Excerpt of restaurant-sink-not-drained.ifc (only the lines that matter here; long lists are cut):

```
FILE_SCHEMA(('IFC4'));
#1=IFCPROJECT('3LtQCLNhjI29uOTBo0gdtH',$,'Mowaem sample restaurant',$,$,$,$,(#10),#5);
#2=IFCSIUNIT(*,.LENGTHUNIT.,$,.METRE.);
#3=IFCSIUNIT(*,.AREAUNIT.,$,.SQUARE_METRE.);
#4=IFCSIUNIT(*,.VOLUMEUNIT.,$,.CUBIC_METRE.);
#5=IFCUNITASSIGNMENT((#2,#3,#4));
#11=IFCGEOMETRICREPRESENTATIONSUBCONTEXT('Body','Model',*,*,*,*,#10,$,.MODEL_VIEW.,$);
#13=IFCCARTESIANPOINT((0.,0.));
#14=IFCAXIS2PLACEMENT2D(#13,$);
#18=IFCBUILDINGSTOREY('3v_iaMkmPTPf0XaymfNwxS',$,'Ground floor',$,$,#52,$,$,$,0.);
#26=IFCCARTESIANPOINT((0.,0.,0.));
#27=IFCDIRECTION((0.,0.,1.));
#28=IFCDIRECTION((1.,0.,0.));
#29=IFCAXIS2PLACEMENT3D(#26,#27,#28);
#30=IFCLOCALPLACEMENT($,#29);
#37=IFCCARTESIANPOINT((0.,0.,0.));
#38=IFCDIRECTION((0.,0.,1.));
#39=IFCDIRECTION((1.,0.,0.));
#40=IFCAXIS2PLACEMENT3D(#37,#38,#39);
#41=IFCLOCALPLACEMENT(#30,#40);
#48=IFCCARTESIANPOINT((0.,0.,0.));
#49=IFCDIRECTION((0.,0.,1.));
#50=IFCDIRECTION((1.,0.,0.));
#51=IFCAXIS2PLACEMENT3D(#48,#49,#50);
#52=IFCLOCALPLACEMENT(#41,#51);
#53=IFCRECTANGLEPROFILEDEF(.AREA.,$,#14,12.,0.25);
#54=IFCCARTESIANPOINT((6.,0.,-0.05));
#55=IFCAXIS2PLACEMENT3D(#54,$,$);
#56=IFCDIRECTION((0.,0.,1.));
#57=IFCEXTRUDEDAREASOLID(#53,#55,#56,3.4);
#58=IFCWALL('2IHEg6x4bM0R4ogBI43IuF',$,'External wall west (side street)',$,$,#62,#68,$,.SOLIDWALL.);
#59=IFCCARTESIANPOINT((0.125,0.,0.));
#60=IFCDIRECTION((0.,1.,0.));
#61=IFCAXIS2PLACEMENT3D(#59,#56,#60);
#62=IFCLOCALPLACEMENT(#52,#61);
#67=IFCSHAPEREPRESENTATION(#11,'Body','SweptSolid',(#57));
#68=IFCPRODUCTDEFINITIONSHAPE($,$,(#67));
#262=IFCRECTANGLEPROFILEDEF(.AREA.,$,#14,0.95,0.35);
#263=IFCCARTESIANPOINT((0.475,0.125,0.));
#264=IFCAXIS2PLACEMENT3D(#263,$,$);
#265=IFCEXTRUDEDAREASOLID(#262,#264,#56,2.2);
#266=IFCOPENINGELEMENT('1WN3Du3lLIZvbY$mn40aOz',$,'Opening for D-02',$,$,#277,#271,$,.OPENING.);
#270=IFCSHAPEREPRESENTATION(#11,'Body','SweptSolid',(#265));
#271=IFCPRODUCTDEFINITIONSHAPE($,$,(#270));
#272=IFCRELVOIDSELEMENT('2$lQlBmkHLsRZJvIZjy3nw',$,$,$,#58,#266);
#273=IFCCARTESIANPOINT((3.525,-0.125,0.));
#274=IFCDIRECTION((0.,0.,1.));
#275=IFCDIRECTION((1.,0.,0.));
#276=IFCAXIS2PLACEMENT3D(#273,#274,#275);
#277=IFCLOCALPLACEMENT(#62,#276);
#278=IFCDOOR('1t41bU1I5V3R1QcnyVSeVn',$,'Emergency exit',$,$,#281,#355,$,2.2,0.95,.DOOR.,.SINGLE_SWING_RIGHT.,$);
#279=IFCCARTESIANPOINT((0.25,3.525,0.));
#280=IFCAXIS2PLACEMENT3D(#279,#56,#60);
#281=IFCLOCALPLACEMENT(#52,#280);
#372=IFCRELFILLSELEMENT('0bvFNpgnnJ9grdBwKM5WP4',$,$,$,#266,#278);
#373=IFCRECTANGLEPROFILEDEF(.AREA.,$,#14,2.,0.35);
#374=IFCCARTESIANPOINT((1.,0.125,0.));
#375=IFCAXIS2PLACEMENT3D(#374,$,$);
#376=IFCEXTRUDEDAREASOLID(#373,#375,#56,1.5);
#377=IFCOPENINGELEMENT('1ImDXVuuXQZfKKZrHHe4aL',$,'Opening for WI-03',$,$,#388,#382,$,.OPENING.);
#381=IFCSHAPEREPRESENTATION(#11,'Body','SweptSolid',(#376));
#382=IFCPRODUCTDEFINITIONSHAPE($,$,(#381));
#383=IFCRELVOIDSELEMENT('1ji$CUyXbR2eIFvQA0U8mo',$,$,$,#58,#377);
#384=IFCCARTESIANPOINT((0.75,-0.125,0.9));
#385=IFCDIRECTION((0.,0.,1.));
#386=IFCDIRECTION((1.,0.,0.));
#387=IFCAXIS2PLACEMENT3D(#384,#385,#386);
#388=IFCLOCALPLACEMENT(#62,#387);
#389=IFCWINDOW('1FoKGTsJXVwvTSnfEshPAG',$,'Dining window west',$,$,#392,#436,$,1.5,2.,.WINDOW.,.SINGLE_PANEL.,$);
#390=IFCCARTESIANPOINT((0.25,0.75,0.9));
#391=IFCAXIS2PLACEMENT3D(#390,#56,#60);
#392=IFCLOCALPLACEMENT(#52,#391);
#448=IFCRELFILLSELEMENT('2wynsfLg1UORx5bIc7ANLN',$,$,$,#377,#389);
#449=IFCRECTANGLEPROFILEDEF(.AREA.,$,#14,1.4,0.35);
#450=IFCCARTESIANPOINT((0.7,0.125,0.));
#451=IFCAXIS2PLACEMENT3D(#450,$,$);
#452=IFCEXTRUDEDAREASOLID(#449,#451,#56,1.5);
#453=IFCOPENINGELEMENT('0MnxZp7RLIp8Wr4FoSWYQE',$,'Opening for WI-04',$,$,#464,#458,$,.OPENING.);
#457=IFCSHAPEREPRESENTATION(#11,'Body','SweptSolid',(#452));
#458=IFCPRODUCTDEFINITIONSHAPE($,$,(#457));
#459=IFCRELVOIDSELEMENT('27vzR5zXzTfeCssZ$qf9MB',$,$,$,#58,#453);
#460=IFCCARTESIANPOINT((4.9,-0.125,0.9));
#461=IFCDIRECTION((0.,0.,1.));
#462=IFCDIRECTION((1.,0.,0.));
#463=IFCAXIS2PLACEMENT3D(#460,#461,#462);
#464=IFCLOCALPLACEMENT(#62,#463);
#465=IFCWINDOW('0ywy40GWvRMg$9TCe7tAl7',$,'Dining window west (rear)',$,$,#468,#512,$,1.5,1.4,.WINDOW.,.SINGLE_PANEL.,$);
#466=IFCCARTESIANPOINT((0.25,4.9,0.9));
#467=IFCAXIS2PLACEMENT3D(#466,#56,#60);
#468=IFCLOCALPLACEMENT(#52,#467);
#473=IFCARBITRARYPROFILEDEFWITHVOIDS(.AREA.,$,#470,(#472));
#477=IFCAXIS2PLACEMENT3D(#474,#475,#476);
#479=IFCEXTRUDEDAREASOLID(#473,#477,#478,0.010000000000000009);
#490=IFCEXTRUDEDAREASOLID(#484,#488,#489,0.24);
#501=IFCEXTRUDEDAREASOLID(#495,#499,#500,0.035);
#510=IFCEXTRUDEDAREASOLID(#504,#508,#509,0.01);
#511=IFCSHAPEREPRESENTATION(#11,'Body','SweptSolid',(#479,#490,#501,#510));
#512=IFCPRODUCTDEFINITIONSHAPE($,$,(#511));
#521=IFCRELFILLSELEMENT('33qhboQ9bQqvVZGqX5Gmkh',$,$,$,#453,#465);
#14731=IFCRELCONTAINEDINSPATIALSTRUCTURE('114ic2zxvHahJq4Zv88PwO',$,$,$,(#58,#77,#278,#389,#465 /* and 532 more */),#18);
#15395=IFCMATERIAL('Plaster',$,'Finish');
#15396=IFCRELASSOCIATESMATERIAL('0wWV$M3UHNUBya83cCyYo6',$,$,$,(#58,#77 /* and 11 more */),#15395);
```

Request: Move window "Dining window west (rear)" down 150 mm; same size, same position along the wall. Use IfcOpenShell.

```python
import numpy as np
import ifcopenshell
import ifcopenshell.api.geometry
import ifcopenshell.util.placement
import ifcopenshell.util.unit

model = ifcopenshell.open("restaurant-sink-not-drained.ifc")
unit_scale = ifcopenshell.util.unit.calculate_unit_scale(model)

window = model.by_guid("0ywy40GWvRMg$9TCe7tAl7")
opening = window.FillsVoids[0].RelatingOpeningElement
dz = -0.15 / unit_scale

shift = np.array([0.0, 0.0, dz])
# The window is not placed relative to its opening, so move both.
for product in (opening, window):
    matrix = ifcopenshell.util.placement.get_local_placement(product.ObjectPlacement)
    matrix[:3, 3] += shift
    ifcopenshell.api.geometry.edit_object_placement(model, product=product, matrix=matrix, is_si=False)

print(f"moved by {dz * unit_scale:+.3f} m")

model.write("restaurant-sink-not-drained-out.ifc")
```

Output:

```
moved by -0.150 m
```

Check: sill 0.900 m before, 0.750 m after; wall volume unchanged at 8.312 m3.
